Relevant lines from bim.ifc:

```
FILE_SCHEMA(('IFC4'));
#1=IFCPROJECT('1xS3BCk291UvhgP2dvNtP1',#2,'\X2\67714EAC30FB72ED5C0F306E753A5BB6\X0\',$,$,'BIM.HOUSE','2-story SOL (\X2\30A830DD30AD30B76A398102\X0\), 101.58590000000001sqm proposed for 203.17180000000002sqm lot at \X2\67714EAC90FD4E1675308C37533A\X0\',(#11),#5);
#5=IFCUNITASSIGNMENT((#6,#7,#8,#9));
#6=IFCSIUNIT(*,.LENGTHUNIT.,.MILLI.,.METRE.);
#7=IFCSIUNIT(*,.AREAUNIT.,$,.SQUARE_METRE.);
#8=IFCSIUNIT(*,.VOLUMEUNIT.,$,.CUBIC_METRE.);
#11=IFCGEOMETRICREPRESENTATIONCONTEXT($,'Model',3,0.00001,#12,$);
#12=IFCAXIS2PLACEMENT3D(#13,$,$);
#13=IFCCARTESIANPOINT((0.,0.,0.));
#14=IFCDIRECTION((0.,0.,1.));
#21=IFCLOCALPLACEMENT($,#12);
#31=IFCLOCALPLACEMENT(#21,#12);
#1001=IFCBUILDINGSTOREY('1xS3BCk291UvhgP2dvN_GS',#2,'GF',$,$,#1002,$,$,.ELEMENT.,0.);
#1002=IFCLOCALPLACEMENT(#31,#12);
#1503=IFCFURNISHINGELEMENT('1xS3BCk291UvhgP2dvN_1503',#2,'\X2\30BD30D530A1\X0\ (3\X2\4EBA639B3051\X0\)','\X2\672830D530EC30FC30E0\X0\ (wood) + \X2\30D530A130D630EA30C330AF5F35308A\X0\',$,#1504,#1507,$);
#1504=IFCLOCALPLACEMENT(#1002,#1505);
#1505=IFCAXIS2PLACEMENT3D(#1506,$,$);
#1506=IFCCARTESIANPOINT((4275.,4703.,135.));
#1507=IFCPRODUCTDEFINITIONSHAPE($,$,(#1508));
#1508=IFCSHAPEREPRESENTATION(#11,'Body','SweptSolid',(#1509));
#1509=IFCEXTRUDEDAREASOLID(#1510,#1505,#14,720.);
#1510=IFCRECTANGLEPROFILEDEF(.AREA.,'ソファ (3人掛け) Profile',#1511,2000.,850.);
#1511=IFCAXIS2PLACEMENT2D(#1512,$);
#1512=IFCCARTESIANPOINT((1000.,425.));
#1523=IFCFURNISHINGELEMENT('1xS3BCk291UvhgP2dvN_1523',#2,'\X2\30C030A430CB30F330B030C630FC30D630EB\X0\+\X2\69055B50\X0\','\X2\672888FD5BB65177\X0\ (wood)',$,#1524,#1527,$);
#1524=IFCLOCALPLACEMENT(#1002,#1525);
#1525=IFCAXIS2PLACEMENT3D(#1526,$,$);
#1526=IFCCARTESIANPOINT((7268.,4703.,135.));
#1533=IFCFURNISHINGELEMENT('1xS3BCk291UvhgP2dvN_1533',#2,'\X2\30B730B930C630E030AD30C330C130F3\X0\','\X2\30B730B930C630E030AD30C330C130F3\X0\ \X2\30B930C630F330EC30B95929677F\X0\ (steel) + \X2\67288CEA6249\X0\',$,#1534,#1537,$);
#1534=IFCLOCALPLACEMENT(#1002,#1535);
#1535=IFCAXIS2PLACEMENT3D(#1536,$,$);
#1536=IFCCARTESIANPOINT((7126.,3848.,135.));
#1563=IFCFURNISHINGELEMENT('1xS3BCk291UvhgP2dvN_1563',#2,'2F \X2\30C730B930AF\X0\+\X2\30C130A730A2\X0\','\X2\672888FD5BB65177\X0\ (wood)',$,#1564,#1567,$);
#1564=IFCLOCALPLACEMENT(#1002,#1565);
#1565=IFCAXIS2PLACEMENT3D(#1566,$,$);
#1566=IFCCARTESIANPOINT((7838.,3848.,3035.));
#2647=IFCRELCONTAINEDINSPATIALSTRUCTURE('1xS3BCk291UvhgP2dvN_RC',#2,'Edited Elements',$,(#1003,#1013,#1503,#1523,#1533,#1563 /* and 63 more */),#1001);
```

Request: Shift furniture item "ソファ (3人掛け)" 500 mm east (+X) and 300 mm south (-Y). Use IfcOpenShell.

```python
import ifcopenshell
import ifcopenshell.api.geometry
import ifcopenshell.util.placement

model = ifcopenshell.open("bim.ifc")

item = model.by_guid("1xS3BCk291UvhgP2dvN_1503")
matrix = ifcopenshell.util.placement.get_local_placement(item.ObjectPlacement)
matrix[0, 3] += 500.0
matrix[1, 3] -= 300.0
ifcopenshell.api.geometry.edit_object_placement(model, product=item, matrix=matrix, is_si=False)

print(ifcopenshell.util.placement.get_local_placement(item.ObjectPlacement).round(3) + 0.0)

model.write("bim_v2.ifc")
```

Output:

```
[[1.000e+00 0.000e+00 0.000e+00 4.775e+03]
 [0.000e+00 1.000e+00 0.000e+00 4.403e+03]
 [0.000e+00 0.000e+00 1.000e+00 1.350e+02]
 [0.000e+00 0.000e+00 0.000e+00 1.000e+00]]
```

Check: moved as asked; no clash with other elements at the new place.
